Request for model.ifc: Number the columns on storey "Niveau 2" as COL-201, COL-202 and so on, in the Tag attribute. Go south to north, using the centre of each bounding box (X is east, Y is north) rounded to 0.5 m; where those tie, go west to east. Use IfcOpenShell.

First a look at what the model holds.

```python
import ifcopenshell
import ifcopenshell.util.element
import ifcopenshell.util.placement

model = ifcopenshell.open("model.ifc")
print(model.schema)
storey = next(s for s in model.by_type("IfcBuildingStorey") if s.Name == "Niveau 2")
columns = [e for e in ifcopenshell.util.element.get_decomposition(storey) if e.is_a("IfcColumn")]
for e in sorted(columns, key=lambda e: e.id()):
    origin = ifcopenshell.util.placement.get_local_placement(e.ObjectPlacement)[:3, 3]
    print(e.id(), e.Tag, e.Name, origin.round(2) + 0.0, sep=" | ")
```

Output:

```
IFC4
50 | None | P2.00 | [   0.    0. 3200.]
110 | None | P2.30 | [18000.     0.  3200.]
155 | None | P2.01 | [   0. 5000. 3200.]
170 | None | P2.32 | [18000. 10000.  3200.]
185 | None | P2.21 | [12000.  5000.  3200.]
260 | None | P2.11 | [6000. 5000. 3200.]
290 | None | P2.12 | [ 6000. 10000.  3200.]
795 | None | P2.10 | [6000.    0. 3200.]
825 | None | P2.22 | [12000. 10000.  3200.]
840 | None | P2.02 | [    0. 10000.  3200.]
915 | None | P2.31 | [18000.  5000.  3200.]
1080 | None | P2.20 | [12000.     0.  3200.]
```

```python
import ifcopenshell
import ifcopenshell.geom
import ifcopenshell.util.element
import ifcopenshell.util.shape

model = ifcopenshell.open("model.ifc")
settings = ifcopenshell.geom.settings()
settings.set("use-world-coords", True)


def centre(element):
    shape = ifcopenshell.geom.create_shape(settings, element)
    return ifcopenshell.util.shape.get_bbox_centroid(shape.geometry)


storey = next(s for s in model.by_type("IfcBuildingStorey") if s.Name == "Niveau 2")
columns = [e for e in ifcopenshell.util.element.get_decomposition(storey) if e.is_a("IfcColumn")]

# Insertion points can sit at a corner or the storey origin, so sort by the geometry (in metres).
centres = {e: centre(e) for e in columns}
columns.sort(key=lambda e: (round(centres[e][1] / 0.5), centres[e][0]))

for i, e in enumerate(columns, start=1):
    number = f"COL-2{i:02d}"
    e.Tag = number
    print(e.id(), number)

model.write("model-out.ifc")
```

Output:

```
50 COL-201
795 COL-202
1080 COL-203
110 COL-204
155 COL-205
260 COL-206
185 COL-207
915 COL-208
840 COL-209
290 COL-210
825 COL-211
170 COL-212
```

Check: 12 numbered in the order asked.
